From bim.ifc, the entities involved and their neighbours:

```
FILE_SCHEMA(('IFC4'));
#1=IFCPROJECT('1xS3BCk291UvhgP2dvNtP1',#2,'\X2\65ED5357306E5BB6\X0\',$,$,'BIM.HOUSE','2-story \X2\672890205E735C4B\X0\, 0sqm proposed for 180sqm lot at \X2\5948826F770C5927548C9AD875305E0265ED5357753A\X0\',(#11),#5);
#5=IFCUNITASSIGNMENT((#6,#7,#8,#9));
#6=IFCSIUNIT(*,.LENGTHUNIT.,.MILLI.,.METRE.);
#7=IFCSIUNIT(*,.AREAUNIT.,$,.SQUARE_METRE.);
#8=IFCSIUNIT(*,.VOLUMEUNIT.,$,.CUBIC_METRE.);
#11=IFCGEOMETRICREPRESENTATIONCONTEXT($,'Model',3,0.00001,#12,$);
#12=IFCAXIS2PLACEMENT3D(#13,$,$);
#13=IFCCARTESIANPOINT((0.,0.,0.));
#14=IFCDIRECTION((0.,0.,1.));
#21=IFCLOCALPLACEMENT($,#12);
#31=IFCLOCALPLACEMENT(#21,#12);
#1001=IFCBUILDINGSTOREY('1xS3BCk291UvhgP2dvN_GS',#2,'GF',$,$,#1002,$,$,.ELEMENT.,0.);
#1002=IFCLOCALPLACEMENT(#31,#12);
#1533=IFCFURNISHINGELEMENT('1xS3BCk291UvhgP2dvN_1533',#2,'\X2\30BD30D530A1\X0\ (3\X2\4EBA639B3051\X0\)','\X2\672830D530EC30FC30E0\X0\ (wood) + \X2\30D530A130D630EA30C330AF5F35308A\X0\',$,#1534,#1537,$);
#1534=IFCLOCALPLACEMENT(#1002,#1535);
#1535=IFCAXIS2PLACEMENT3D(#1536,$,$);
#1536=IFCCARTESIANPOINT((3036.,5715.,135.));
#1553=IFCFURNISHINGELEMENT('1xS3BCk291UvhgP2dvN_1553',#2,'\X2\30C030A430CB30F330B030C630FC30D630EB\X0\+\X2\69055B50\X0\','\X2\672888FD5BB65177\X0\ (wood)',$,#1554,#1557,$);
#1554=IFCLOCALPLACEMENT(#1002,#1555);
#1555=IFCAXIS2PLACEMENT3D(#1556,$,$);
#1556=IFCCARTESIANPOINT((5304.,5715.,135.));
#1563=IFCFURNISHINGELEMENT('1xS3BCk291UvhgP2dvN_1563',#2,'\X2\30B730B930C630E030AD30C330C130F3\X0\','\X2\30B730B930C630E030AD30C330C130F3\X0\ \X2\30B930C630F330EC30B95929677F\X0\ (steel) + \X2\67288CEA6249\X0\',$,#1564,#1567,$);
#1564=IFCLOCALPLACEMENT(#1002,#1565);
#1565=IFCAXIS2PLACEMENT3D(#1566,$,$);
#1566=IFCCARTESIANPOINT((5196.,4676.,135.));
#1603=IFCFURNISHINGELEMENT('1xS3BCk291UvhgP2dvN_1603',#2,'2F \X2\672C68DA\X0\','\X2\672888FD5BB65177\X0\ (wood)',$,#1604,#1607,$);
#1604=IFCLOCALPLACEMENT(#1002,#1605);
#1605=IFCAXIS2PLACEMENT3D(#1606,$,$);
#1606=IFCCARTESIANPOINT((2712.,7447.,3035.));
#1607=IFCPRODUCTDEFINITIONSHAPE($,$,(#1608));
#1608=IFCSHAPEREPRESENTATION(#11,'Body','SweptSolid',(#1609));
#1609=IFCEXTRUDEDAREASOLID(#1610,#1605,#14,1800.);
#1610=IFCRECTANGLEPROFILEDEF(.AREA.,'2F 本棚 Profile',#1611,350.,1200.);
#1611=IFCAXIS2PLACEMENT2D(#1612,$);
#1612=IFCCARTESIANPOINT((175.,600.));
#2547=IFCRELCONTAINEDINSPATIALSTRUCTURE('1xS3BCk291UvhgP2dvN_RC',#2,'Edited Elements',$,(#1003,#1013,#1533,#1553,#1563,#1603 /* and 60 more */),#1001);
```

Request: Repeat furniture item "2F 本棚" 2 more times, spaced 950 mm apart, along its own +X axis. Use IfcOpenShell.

```python
import ifcopenshell
import ifcopenshell.api.geometry
import ifcopenshell.api.root
import ifcopenshell.util.element
import ifcopenshell.util.placement

model = ifcopenshell.open("bim.ifc")


def reuse_history(source, copy):
    """copy_class also copies each property set's owner history, people and application; keep the originals."""
    for rel in copy.IsDefinedBy:
        if rel.is_a("IfcRelDefinesByProperties") and (history := rel.RelatingPropertyDefinition.OwnerHistory):
            rel.RelatingPropertyDefinition.OwnerHistory = source.OwnerHistory
            ifcopenshell.util.element.remove_deep2(model, history)


source = model.by_guid("1xS3BCk291UvhgP2dvN_1603")
base = ifcopenshell.util.placement.get_local_placement(source.ObjectPlacement)
step = base[:3, 0] * 950.0

for i in range(1, 3):
    copy = ifcopenshell.api.root.copy_class(model, product=source)
    copy.Representation = ifcopenshell.util.element.copy_deep(
        model, source.Representation, exclude=["IfcGeometricRepresentationContext", "IfcRepresentationMap"]
    )
    reuse_history(source, copy)
    matrix = base.copy()
    matrix[:3, 3] += i * step
    print("added at", matrix[:3, 3].round(3) + 0.0)
    ifcopenshell.api.geometry.edit_object_placement(model, product=copy, matrix=matrix, is_si=False)

model.write("bim_updated.ifc")
```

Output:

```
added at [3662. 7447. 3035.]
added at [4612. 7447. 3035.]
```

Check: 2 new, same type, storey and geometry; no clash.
